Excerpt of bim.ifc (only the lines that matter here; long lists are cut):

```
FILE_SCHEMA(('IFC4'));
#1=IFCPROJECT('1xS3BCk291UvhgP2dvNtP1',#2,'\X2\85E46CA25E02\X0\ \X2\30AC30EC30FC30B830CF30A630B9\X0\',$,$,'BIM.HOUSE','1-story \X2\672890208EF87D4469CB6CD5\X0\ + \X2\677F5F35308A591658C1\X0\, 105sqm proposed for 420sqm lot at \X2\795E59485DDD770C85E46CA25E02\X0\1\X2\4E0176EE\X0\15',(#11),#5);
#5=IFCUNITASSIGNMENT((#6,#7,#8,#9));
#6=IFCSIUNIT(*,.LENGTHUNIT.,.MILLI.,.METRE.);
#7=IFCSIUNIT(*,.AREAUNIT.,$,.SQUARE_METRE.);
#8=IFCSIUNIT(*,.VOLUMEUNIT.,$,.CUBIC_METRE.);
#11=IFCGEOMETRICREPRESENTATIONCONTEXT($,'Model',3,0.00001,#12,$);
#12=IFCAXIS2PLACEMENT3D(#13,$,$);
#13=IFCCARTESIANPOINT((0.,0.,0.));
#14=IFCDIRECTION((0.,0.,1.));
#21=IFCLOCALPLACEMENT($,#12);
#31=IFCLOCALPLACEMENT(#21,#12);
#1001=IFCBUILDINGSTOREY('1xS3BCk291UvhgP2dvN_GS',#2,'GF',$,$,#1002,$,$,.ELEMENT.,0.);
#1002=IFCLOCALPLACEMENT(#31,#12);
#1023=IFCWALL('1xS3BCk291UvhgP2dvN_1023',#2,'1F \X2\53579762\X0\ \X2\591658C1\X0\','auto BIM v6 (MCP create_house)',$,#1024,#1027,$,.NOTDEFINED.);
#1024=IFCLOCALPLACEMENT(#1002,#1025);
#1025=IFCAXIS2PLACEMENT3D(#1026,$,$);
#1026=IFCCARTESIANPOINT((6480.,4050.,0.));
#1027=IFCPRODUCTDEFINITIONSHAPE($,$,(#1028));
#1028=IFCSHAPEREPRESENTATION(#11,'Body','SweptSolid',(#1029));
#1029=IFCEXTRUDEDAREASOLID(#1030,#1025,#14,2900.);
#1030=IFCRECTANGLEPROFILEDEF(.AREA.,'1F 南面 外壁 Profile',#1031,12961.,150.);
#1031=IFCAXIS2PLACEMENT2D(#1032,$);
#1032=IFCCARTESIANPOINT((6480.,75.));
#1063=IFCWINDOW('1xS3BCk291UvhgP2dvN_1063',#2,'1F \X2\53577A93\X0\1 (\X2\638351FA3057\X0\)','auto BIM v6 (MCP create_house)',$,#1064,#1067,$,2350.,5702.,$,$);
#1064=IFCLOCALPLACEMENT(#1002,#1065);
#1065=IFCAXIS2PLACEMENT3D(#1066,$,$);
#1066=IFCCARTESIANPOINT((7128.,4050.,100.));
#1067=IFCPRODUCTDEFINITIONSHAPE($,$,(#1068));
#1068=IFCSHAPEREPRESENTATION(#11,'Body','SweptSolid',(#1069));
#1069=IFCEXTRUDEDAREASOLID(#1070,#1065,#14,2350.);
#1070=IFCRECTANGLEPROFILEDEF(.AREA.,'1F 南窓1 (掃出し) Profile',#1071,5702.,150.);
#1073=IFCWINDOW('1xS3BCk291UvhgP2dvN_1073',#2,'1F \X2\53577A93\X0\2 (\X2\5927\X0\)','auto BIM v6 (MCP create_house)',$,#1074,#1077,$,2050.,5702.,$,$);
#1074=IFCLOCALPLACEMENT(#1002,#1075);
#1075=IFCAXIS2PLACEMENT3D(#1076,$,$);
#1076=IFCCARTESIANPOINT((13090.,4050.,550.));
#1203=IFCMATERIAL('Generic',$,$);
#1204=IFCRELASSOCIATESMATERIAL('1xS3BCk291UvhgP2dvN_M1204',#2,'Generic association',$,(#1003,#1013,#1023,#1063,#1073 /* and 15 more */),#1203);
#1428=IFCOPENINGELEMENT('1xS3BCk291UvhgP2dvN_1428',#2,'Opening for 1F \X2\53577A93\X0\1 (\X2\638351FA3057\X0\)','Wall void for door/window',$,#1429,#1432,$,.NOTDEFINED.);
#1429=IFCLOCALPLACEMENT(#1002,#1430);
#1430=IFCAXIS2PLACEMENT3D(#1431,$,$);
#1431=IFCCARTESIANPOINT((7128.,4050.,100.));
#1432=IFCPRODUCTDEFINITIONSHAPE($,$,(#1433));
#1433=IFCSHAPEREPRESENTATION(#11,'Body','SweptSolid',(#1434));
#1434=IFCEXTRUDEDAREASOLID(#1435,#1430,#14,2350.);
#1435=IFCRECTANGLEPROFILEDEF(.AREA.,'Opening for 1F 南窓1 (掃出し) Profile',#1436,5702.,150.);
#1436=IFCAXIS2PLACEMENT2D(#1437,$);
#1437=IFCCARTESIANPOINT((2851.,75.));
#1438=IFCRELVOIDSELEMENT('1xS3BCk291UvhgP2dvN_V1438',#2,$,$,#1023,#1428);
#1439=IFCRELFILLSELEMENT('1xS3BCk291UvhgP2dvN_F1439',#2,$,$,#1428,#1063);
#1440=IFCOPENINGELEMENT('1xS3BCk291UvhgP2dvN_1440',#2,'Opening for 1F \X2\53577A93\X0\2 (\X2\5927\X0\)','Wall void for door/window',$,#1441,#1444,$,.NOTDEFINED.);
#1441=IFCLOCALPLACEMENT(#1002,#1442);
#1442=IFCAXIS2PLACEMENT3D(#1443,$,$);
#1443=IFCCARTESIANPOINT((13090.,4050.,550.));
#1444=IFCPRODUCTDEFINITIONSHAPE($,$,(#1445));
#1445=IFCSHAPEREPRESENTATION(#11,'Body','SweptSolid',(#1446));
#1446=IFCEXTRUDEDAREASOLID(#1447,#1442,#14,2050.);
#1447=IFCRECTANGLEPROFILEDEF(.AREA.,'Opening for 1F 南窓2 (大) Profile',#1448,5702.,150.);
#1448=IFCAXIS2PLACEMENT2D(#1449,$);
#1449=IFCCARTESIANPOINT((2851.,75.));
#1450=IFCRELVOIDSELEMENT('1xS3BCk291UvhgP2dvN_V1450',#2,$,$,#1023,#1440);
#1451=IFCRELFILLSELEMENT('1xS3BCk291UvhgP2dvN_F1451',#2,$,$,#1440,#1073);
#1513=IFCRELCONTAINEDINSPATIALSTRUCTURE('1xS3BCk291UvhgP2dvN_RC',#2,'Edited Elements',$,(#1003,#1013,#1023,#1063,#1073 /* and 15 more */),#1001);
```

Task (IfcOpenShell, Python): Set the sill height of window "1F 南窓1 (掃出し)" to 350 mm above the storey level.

```python
import numpy as np
import ifcopenshell
import ifcopenshell.api.geometry
import ifcopenshell.geom
import ifcopenshell.util.element
import ifcopenshell.util.placement
import ifcopenshell.util.shape
import ifcopenshell.util.unit

model = ifcopenshell.open("bim.ifc")
unit_scale = ifcopenshell.util.unit.calculate_unit_scale(model)

window = model.by_guid("1xS3BCk291UvhgP2dvN_1063")
opening = window.FillsVoids[0].RelatingOpeningElement
storey = ifcopenshell.util.element.get_container(window, ifc_class="IfcBuildingStorey")
level = ifcopenshell.util.placement.get_local_placement(storey.ObjectPlacement)[2, 3]

# The opening's origin need not be at the sill, so measure its lowest point.
shape = ifcopenshell.geom.create_shape(ifcopenshell.geom.settings(), opening)
bottom = ifcopenshell.util.shape.get_shape_bottom_elevation(shape, shape.geometry) / unit_scale
dz = level + 350.0 - bottom

shift = np.array([0.0, 0.0, dz])
# The window is not placed relative to its opening, so move both.
for product in (opening, window):
    matrix = ifcopenshell.util.placement.get_local_placement(product.ObjectPlacement)
    matrix[:3, 3] += shift
    ifcopenshell.api.geometry.edit_object_placement(model, product=product, matrix=matrix, is_si=False)

print(f"moved by {dz * unit_scale:+.3f} m")

model.write("bim_v2.ifc")
```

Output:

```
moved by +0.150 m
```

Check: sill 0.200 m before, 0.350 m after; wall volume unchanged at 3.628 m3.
